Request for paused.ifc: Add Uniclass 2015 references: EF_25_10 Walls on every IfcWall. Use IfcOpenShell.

First a look at what the model holds.

```python
import ifcopenshell

model = ifcopenshell.open("paused.ifc")
print(model.schema)
print("classifications:", [c.Name for c in model.by_type("IfcClassification")])
for ifc_class in ("IfcDoor", "IfcRoof", "IfcStair", "IfcWall", "IfcWindow"):
    print(ifc_class, len(model.by_type(ifc_class)))
```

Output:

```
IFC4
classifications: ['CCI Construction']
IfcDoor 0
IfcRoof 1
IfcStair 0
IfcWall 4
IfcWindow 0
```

```python
import ifcopenshell
import ifcopenshell.api.classification

model = ifcopenshell.open("paused.ifc")

system = ifcopenshell.api.classification.add_classification(model, classification="Uniclass 2015")

codes = {
    "IfcWall": ("EF_25_10", "Walls"),
}
for ifc_class, (code, name) in codes.items():
    products = model.by_type(ifc_class)
    ifcopenshell.api.classification.add_reference(
        model, products=products, classification=system, identification=code, name=name
    )
    print(code, len(products))

model.write("paused-out.ifc")
```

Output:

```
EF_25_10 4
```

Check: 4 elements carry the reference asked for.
